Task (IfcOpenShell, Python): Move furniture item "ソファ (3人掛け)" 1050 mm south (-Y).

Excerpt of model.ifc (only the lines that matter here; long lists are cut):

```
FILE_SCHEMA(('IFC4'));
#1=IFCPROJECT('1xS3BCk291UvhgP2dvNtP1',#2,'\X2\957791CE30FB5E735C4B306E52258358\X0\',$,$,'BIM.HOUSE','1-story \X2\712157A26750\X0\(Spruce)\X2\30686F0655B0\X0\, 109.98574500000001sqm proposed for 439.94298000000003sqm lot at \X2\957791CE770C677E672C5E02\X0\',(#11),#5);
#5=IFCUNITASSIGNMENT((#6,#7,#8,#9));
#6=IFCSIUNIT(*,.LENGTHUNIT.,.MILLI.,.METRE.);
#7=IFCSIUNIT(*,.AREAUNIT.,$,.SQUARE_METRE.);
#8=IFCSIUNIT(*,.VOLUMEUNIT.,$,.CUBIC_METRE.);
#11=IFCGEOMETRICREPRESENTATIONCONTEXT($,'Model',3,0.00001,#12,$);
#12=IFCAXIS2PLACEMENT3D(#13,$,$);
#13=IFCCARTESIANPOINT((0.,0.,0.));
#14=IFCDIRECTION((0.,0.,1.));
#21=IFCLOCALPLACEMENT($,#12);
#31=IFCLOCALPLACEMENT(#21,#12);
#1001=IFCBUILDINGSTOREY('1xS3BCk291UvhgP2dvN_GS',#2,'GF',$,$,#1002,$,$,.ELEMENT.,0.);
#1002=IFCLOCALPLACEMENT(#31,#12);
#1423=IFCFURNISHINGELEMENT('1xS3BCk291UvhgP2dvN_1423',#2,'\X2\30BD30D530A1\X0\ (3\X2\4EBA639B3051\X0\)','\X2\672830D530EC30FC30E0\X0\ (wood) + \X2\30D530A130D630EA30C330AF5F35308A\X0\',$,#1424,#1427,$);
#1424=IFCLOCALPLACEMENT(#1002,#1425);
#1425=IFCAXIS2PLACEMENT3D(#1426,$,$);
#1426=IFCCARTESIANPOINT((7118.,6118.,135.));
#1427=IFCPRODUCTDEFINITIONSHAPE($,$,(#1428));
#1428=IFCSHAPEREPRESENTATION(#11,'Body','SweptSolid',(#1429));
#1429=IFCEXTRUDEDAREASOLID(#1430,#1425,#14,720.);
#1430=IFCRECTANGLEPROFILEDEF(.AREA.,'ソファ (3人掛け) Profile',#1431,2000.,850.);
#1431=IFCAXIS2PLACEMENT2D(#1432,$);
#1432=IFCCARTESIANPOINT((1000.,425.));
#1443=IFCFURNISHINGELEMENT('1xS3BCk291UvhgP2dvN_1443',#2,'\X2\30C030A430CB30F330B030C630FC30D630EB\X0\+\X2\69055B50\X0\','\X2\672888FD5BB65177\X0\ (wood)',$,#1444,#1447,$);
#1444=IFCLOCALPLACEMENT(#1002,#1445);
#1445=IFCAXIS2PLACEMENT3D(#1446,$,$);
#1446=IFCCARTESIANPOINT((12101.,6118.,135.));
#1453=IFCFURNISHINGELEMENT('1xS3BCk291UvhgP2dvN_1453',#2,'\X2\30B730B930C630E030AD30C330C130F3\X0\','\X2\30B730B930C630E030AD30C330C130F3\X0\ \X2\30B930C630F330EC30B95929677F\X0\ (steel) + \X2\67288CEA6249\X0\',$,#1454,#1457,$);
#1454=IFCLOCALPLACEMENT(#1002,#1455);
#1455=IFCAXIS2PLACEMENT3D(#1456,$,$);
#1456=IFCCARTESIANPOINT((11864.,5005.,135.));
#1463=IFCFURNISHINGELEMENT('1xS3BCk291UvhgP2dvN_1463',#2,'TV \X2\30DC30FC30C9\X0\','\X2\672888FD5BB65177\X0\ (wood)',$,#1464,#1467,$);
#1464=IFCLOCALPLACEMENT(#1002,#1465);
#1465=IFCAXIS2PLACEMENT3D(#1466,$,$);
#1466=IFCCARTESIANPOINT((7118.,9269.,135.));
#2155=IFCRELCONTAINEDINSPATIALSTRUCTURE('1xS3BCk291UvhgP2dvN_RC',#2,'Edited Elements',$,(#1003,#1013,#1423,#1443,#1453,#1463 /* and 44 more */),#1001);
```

```python
import ifcopenshell
import ifcopenshell.api.geometry
import ifcopenshell.util.placement

model = ifcopenshell.open("model.ifc")

item = model.by_guid("1xS3BCk291UvhgP2dvN_1423")
matrix = ifcopenshell.util.placement.get_local_placement(item.ObjectPlacement)
matrix[1, 3] -= 1050.0
ifcopenshell.api.geometry.edit_object_placement(model, product=item, matrix=matrix, is_si=False)

print(ifcopenshell.util.placement.get_local_placement(item.ObjectPlacement).round(3) + 0.0)

model.write("model_updated.ifc")
```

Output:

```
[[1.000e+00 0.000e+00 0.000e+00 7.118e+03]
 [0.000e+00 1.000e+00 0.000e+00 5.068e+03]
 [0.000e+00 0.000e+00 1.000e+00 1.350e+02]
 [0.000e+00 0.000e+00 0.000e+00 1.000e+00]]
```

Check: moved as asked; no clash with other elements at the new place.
